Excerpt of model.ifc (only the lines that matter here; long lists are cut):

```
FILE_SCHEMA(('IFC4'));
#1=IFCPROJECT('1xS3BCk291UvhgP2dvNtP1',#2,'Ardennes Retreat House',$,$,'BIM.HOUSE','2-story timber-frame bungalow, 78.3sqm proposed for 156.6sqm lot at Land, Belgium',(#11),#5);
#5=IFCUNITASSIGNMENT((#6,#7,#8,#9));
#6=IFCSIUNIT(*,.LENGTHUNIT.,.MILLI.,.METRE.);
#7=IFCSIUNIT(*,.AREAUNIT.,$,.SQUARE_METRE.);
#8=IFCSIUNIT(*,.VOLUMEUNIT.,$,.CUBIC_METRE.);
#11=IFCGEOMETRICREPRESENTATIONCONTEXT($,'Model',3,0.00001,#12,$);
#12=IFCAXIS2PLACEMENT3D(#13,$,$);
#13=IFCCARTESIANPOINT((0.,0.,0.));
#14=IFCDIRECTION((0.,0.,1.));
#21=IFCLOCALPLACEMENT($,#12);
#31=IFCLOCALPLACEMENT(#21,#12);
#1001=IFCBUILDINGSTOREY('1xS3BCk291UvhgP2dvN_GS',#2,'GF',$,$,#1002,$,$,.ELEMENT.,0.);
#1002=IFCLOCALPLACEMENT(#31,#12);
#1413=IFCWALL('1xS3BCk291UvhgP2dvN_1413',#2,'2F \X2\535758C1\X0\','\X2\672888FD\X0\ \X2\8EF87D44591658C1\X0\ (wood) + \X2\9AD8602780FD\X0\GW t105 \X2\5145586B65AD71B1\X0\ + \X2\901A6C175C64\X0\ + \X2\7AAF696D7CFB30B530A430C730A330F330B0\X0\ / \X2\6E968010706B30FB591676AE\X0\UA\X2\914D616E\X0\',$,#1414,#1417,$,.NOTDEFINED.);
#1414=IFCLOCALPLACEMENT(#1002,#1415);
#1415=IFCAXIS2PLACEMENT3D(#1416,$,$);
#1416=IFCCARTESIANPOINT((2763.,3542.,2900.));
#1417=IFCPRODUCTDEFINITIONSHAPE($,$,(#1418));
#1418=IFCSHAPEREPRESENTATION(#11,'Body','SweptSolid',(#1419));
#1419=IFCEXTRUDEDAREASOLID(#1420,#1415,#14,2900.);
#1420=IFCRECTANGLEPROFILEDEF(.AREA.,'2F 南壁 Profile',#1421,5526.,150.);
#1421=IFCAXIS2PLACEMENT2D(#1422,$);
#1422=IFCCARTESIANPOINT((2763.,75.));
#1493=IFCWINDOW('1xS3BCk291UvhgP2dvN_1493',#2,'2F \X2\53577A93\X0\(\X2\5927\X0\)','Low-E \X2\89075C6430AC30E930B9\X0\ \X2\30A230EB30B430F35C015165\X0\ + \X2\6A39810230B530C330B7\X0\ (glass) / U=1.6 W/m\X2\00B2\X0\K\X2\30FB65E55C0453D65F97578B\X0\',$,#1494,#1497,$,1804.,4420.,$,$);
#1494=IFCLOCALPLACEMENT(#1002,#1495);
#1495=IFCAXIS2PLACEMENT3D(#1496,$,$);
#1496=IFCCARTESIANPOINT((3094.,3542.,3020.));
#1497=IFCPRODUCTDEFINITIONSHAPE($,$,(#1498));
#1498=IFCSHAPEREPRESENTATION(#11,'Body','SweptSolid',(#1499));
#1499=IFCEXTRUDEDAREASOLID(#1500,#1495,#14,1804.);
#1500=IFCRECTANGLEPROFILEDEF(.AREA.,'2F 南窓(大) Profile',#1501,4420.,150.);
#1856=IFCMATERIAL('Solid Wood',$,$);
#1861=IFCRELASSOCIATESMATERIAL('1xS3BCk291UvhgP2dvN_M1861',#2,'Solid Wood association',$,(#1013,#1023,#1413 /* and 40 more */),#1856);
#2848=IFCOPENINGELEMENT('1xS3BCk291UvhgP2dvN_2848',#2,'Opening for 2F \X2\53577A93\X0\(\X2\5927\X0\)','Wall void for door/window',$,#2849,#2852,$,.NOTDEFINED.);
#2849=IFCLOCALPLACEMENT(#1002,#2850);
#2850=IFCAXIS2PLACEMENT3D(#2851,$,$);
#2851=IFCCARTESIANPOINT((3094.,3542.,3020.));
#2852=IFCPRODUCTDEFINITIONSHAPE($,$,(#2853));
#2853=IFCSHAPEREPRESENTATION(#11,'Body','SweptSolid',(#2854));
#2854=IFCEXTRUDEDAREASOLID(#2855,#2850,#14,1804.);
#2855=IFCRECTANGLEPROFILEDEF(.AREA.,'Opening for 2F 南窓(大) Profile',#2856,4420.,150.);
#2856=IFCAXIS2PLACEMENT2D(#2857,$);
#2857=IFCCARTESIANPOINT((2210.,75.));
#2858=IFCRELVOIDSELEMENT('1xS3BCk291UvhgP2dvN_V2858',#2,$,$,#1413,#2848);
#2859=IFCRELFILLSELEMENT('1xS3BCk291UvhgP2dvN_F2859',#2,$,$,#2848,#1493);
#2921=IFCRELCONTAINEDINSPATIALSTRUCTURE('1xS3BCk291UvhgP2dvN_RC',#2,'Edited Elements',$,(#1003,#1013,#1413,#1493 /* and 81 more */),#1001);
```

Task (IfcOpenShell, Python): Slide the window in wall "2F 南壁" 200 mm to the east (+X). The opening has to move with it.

```python
import ifcopenshell
import ifcopenshell.api.geometry
import ifcopenshell.util.placement

model = ifcopenshell.open("model.ifc")

window = model.by_guid("1xS3BCk291UvhgP2dvN_1493")
opening = window.FillsVoids[0].RelatingOpeningElement
wall = opening.VoidsElements[0].RelatingBuildingElement

wall_matrix = ifcopenshell.util.placement.get_local_placement(wall.ObjectPlacement)
shift = wall_matrix[:3, 0] * 200.0
before = ifcopenshell.util.placement.get_local_placement(window.ObjectPlacement)[:3, 3].copy()

# The window is not placed relative to its opening, so move both.
for product in (opening, window):
    matrix = ifcopenshell.util.placement.get_local_placement(product.ObjectPlacement)
    matrix[:3, 3] += shift
    ifcopenshell.api.geometry.edit_object_placement(model, product=product, matrix=matrix, is_si=False)

after = ifcopenshell.util.placement.get_local_placement(window.ObjectPlacement)[:3, 3]
print("window moved by", (after - before).round(3) + 0.0)

model.write("model_edited.ifc")
```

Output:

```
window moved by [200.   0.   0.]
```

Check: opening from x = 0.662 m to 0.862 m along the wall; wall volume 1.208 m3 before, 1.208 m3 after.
